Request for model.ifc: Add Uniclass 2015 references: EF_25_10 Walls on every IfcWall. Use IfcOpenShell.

First a look at what the model holds.

```python
import ifcopenshell

model = ifcopenshell.open("model.ifc")
print(model.schema)
print("classifications:", [c.Name for c in model.by_type("IfcClassification")])
for ifc_class in ("IfcDoor", "IfcRoof", "IfcStair", "IfcWall", "IfcWindow"):
    print(ifc_class, len(model.by_type(ifc_class)))
```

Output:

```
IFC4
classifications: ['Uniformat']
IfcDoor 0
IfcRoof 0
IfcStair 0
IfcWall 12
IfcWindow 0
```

```python
import ifcopenshell
import ifcopenshell.api.classification

model = ifcopenshell.open("model.ifc")

system = ifcopenshell.api.classification.add_classification(model, classification="Uniclass 2015")

codes = {
    "IfcWall": ("EF_25_10", "Walls"),
}
for ifc_class, (code, name) in codes.items():
    products = model.by_type(ifc_class)
    ifcopenshell.api.classification.add_reference(
        model, products=products, classification=system, identification=code, name=name
    )
    print(code, len(products))

model.write("model_updated.ifc")
```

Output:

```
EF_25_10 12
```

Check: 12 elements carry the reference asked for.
